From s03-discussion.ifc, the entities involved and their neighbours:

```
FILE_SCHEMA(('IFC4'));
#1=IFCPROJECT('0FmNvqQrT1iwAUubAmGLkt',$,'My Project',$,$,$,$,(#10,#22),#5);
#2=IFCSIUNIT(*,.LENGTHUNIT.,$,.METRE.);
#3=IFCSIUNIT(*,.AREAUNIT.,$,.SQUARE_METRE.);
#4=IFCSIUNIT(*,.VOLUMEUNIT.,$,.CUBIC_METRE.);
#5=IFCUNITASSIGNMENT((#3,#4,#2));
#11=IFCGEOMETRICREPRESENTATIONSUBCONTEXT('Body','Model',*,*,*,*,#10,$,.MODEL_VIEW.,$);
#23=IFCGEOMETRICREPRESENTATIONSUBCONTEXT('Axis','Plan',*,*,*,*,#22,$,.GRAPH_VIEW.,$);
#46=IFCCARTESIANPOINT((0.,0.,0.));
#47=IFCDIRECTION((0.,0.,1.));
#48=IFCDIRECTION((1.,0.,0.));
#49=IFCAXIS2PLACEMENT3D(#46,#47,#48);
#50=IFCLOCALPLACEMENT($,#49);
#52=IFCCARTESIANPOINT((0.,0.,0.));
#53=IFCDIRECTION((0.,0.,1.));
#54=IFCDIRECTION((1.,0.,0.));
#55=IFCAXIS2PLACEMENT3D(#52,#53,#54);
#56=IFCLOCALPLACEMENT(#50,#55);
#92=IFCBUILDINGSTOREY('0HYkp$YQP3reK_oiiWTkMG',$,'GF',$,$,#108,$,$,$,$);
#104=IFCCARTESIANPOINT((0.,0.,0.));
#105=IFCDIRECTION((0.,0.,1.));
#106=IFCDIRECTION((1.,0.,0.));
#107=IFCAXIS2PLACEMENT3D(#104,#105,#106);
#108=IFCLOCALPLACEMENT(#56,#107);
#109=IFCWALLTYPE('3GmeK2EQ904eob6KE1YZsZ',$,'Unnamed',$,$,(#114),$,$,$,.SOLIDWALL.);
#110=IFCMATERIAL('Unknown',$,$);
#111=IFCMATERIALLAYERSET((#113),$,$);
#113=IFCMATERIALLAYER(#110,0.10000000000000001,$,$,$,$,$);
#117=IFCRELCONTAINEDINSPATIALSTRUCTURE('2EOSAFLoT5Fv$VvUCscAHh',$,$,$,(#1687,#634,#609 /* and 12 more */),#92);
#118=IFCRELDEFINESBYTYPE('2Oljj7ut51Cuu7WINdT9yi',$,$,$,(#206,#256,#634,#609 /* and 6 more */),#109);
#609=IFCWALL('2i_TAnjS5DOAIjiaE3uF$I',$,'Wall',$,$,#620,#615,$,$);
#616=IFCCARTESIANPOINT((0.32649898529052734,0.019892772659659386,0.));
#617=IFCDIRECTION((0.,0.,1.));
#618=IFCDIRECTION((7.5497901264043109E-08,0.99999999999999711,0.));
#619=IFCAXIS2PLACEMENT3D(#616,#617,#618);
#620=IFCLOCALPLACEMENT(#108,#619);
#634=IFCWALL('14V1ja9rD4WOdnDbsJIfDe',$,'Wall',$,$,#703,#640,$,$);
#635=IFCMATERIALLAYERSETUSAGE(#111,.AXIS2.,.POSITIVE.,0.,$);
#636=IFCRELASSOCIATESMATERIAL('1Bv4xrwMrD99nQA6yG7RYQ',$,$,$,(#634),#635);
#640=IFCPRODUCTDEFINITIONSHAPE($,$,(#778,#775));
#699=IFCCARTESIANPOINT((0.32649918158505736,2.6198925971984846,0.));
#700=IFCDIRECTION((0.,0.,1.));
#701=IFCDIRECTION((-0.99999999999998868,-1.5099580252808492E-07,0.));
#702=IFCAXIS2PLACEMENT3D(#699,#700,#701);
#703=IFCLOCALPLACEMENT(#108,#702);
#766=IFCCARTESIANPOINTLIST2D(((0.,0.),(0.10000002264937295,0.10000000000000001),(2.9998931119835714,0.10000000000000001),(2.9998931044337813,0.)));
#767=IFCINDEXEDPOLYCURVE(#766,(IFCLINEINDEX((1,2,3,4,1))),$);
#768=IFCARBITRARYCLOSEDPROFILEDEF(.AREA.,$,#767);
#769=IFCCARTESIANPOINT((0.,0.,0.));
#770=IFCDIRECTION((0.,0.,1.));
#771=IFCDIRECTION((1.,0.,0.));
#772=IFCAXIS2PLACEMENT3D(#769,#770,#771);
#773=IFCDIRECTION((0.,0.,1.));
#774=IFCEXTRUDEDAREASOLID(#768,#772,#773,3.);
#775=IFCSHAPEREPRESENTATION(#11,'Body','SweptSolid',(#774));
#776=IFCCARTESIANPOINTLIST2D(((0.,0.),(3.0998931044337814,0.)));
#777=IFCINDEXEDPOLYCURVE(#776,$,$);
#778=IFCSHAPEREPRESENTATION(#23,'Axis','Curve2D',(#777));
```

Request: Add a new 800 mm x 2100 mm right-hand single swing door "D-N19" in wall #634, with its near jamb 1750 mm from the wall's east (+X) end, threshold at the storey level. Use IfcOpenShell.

```python
import numpy as np
import ifcopenshell
import ifcopenshell.api.feature
import ifcopenshell.api.geometry
import ifcopenshell.api.root
import ifcopenshell.api.spatial
import ifcopenshell.geom
import ifcopenshell.util.element
import ifcopenshell.util.placement
import ifcopenshell.util.representation
import ifcopenshell.util.shape
import ifcopenshell.util.unit

model = ifcopenshell.open("s03-discussion.ifc")
unit_scale = ifcopenshell.util.unit.calculate_unit_scale(model)
settings = ifcopenshell.geom.settings()


def volume(element):
    """Net volume in cubic metres, openings subtracted."""
    shape = ifcopenshell.geom.create_shape(settings, element)
    return ifcopenshell.util.shape.get_volume(shape.geometry)


wall = model.by_guid("14V1ja9rD4WOdnDbsJIfDe")
storey = ifcopenshell.util.element.get_container(wall, ifc_class="IfcBuildingStorey")
context = ifcopenshell.util.representation.get_context(model, "Model", "Body", "MODEL_VIEW")
before = volume(wall)

width, height, from_end, sill = 0.8, 2.1, 1.75, 0.0  # metres

# The wall runs along its own X axis, and the end named is its -X end.
wall_shape = ifcopenshell.geom.create_shape(settings, wall)
x, y, z = ifcopenshell.util.shape.get_vertices(wall_shape.geometry).T
start = x.min() + from_end
face, thickness = float(y.min()), float(y.max() - y.min())
wall_matrix = ifcopenshell.util.placement.get_local_placement(wall.ObjectPlacement)
level = ifcopenshell.util.placement.get_local_placement(storey.ObjectPlacement)[2, 3]


def in_wall(x, y):
    """Placement at x, y metres in the wall's axes, at sill height."""
    matrix = wall_matrix.copy()
    matrix[:, 3] = wall_matrix @ np.array([x / unit_scale, y / unit_scale, 0.0, 1.0])
    matrix[2, 3] = level + sill / unit_scale
    return matrix


# Opening: a box that overshoots both wall faces by 50 mm.
opening = ifcopenshell.api.root.create_entity(model, ifc_class="IfcOpeningElement", predefined_type="OPENING")
box = ifcopenshell.api.geometry.add_wall_representation(
    model, context=context, length=width, height=height, thickness=thickness + 0.1
)
ifcopenshell.api.geometry.assign_representation(model, product=opening, representation=box)
ifcopenshell.api.geometry.edit_object_placement(model, product=opening, matrix=in_wall(start, face - 0.05), is_si=False)
ifcopenshell.api.feature.add_feature(model, feature=opening, element=wall)

door = ifcopenshell.api.root.create_entity(model, ifc_class="IfcDoor", name="D-N19", predefined_type="DOOR")
door.OverallWidth, door.OverallHeight = width / unit_scale, height / unit_scale
door.OperationType = "SINGLE_SWING_RIGHT"
body = ifcopenshell.api.geometry.add_door_representation(
    model,
    context=context,
    overall_width=door.OverallWidth,
    overall_height=door.OverallHeight,
    operation_type="SINGLE_SWING_RIGHT",
    lining_properties={"LiningDepth": thickness / unit_scale, "ThresholdDepth": thickness / unit_scale},
)
ifcopenshell.api.geometry.assign_representation(model, product=door, representation=body)
ifcopenshell.api.spatial.assign_container(model, products=[door], relating_structure=storey)
ifcopenshell.api.feature.add_filling(model, opening=opening, element=door)

# The lining spans the wall, so the door starts at the wall face.
ifcopenshell.api.geometry.edit_object_placement(model, product=door, matrix=in_wall(start, face), is_si=False)

after = volume(wall)

print(f"wall volume {before:.3f} -> {after:.3f} m3")

model.write("s03-discussion_rev.ifc")
```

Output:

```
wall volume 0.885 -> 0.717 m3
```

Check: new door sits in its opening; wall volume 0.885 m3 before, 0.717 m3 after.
